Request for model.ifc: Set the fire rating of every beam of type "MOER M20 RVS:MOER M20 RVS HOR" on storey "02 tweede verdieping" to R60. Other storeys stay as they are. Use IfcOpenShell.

First a look at what the model holds.

```python
import ifcopenshell
import ifcopenshell.util.element

model = ifcopenshell.open("model.ifc")
print(model.schema)
storey = next(s for s in model.by_type("IfcBuildingStorey") if s.Name == "02 tweede verdieping")
beams = [e for e in ifcopenshell.util.element.get_decomposition(storey) if e.is_a("IfcBeam")]
seen = {}
for e in beams:
    element_type = ifcopenshell.util.element.get_type(e)
    key = (element_type.Name if element_type != e and element_type else None, ifcopenshell.util.element.get_pset(e, "Pset_BeamCommon", "FireRating"))
    seen[key] = seen.get(key, 0) + 1
for (name, value), count in sorted(seen.items(), key=str):
    print(count, "x", name, "|", value)
```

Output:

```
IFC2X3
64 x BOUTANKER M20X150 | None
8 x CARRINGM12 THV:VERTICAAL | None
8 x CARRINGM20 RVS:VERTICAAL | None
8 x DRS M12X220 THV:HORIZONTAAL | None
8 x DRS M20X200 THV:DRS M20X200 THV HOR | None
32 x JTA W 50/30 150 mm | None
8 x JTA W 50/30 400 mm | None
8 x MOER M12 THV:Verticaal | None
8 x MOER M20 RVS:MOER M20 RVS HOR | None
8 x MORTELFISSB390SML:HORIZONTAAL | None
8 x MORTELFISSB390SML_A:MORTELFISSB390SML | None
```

```python
import ifcopenshell
import ifcopenshell.api.pset
import ifcopenshell.util.element

model = ifcopenshell.open("model.ifc")

storey = next(s for s in model.by_type("IfcBuildingStorey") if s.Name == "02 tweede verdieping")
beams = [e for e in ifcopenshell.util.element.get_decomposition(storey) if e.is_a("IfcBeam")]

count = 0
for e in beams:
    element_type = ifcopenshell.util.element.get_type(e)
    if element_type in (None, e) or element_type.Name != "MOER M20 RVS:MOER M20 RVS HOR":
        continue
    # add_pset returns the element's existing set when there is one.
    pset = ifcopenshell.api.pset.add_pset(model, product=e, name="Pset_BeamCommon")
    ifcopenshell.api.pset.edit_pset(model, pset=pset, properties={"FireRating": "R60"})
    count += 1

print(count, "beams updated")

model.write("model_rev.ifc")
```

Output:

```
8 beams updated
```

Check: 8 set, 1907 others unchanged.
